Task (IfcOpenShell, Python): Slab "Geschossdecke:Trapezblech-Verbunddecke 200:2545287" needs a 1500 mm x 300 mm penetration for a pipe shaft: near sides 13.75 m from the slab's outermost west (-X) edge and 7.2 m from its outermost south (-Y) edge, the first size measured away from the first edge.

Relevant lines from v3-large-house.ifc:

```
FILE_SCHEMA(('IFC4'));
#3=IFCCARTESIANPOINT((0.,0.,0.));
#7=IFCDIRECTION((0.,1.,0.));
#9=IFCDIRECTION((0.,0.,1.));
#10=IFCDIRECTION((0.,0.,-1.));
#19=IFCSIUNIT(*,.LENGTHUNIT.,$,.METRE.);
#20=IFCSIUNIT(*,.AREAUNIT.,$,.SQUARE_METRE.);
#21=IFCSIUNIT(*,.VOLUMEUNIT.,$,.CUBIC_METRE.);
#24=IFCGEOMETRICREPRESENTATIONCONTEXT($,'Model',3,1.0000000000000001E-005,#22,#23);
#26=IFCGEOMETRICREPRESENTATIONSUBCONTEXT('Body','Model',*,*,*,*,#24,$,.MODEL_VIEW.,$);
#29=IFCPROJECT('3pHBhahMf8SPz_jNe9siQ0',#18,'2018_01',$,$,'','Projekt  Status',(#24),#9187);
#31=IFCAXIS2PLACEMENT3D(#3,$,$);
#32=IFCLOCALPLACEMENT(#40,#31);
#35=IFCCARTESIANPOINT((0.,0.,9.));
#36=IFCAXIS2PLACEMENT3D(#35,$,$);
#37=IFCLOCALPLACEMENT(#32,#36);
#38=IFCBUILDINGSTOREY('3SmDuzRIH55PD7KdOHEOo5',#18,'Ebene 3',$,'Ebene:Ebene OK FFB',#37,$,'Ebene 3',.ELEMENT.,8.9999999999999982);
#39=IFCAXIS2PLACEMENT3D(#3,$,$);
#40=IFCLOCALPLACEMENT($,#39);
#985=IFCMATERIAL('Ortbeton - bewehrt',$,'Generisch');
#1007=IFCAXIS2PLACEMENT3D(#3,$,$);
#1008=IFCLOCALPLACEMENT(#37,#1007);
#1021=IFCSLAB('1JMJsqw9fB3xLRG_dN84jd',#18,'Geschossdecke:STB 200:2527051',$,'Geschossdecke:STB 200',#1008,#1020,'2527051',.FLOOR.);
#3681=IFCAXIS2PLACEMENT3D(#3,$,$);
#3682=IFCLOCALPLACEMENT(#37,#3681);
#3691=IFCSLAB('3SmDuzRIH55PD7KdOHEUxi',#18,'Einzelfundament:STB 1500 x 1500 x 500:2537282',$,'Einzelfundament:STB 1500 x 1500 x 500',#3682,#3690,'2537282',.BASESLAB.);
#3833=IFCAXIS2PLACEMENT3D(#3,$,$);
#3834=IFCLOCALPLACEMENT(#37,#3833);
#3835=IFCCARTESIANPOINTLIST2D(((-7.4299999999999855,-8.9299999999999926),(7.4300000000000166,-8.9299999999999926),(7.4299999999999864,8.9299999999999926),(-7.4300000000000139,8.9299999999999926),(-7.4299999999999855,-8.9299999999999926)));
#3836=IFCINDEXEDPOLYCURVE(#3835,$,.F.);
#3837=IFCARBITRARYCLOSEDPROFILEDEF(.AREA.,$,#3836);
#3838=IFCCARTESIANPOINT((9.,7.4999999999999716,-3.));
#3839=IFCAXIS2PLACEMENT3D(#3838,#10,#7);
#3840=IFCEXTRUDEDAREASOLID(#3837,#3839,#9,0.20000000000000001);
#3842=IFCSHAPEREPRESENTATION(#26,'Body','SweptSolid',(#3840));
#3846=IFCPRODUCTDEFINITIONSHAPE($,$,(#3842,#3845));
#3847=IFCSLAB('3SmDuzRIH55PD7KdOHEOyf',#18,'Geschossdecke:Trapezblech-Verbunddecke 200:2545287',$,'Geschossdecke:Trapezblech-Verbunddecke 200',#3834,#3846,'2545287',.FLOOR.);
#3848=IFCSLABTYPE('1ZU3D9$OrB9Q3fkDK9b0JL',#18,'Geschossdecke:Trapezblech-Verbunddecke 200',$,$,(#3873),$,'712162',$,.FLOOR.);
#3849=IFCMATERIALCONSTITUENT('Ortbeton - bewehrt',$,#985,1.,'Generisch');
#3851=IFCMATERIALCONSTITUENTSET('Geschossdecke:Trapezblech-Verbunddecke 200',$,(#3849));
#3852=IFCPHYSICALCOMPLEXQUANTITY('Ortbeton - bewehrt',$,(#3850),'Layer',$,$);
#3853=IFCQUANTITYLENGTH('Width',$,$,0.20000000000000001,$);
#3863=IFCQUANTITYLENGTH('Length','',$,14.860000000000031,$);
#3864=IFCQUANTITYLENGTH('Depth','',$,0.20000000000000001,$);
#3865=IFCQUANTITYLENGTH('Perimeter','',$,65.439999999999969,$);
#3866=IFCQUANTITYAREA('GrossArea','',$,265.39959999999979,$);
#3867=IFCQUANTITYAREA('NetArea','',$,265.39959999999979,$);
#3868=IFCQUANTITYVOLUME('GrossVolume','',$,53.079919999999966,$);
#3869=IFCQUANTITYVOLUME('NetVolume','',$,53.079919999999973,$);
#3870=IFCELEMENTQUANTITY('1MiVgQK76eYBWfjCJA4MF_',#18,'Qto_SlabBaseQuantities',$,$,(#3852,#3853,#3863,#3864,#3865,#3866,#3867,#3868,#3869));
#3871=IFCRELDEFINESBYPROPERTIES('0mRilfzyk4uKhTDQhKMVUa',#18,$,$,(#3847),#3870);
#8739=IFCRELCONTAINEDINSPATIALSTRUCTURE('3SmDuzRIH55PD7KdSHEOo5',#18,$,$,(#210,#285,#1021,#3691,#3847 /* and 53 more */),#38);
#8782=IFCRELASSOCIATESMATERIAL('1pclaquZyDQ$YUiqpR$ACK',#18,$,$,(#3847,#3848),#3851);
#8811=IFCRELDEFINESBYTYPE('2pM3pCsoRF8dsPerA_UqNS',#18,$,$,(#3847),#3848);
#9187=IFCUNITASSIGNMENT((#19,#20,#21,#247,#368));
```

```python
import numpy as np
import ifcopenshell
import ifcopenshell.api.feature
import ifcopenshell.api.geometry
import ifcopenshell.api.pset
import ifcopenshell.api.root
import ifcopenshell.geom
import ifcopenshell.util.element
import ifcopenshell.util.placement
import ifcopenshell.util.representation
import ifcopenshell.util.shape
import ifcopenshell.util.unit

model = ifcopenshell.open("v3-large-house.ifc")
unit_scale = ifcopenshell.util.unit.calculate_unit_scale(model)
area_scale = ifcopenshell.util.unit.calculate_unit_scale(model, "AREAUNIT")
volume_scale = ifcopenshell.util.unit.calculate_unit_scale(model, "VOLUMEUNIT")
settings = ifcopenshell.geom.settings()


def volume(element):
    """Net volume in cubic metres, openings subtracted."""
    shape = ifcopenshell.geom.create_shape(settings, element)
    return ifcopenshell.util.shape.get_volume(shape.geometry)


slab = model.by_guid("3SmDuzRIH55PD7KdOHEOyf")
before = volume(slab)

# Extent in the slab's own axes, in metres. The edges named are its -X and -Y sides.
slab_shape = ifcopenshell.geom.create_shape(settings, slab)
vertices = ifcopenshell.util.shape.get_vertices(slab_shape.geometry)
x_min, y_min, bottom = vertices.min(axis=0)
top = vertices[:, 2].max()

opening = ifcopenshell.api.root.create_entity(model, ifc_class="IfcOpeningElement", name="Pipe shaft opening", predefined_type="OPENING")
context = ifcopenshell.util.representation.get_context(model, "Model", "Body", "MODEL_VIEW")
width, depth = 1.5, 0.3
outline = [(0.0, 0.0), (width, 0.0), (width, depth), (0.0, depth), (0.0, 0.0)]
# Overshoot both faces by 50 mm so the cut is clean.
shape = ifcopenshell.api.geometry.add_slab_representation(
    model, context=context, depth=top - bottom + 0.1, polyline=outline
)
ifcopenshell.api.geometry.assign_representation(model, product=opening, representation=shape)

matrix = ifcopenshell.util.placement.get_local_placement(slab.ObjectPlacement)
matrix[:, 3] = matrix @ np.append(np.array([x_min + 13.75, y_min + 7.2, bottom - 0.05]) / unit_scale, 1.0)
ifcopenshell.api.geometry.edit_object_placement(model, product=opening, matrix=matrix, is_si=False)
ifcopenshell.api.feature.add_feature(model, feature=opening, element=slab)

after = volume(slab)

# Update the slab's stored quantities.
qto = model.by_id(ifcopenshell.util.element.get_pset(slab, "Qto_SlabBaseQuantities", should_inherit=False)["id"])
ifcopenshell.api.pset.edit_qto(model, qto=qto, properties={
    "NetArea": after / (top - bottom) / area_scale,
    "NetVolume": after / volume_scale,
})

print(f"slab volume {before:.3f} -> {after:.3f} m3")

model.write("v3-large-house_updated.ifc")
```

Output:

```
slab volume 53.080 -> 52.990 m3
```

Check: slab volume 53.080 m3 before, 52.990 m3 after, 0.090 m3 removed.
